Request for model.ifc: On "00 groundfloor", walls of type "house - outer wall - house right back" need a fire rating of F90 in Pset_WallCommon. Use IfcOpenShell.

First a look at what the model holds.

```python
import ifcopenshell
import ifcopenshell.util.element

model = ifcopenshell.open("model.ifc")
print(model.schema)
storey = next(s for s in model.by_type("IfcBuildingStorey") if s.Name == "00 groundfloor")
walls = [e for e in ifcopenshell.util.element.get_decomposition(storey) if e.is_a("IfcWall")]
seen = {}
for e in walls:
    element_type = ifcopenshell.util.element.get_type(e)
    key = (element_type.Name if element_type != e and element_type else None, ifcopenshell.util.element.get_pset(e, "Pset_WallCommon", "FireRating"))
    seen[key] = seen.get(key, 0) + 1
for (name, value), count in sorted(seen.items(), key=str):
    print(count, "x", name, "|", value)
```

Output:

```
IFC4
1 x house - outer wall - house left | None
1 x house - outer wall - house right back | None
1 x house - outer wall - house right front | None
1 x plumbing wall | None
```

```python
import ifcopenshell
import ifcopenshell.api.pset
import ifcopenshell.util.element

model = ifcopenshell.open("model.ifc")

storey = next(s for s in model.by_type("IfcBuildingStorey") if s.Name == "00 groundfloor")
walls = [e for e in ifcopenshell.util.element.get_decomposition(storey) if e.is_a("IfcWall")]

count = 0
for e in walls:
    element_type = ifcopenshell.util.element.get_type(e)
    if element_type in (None, e) or element_type.Name != "house - outer wall - house right back":
        continue
    # add_pset returns the element's existing set when there is one.
    pset = ifcopenshell.api.pset.add_pset(model, product=e, name="Pset_WallCommon")
    ifcopenshell.api.pset.edit_pset(model, pset=pset, properties={"FireRating": "F90"})
    count += 1

print(count, "walls updated")

model.write("model_edited.ifc")
```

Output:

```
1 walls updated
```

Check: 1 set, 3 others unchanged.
